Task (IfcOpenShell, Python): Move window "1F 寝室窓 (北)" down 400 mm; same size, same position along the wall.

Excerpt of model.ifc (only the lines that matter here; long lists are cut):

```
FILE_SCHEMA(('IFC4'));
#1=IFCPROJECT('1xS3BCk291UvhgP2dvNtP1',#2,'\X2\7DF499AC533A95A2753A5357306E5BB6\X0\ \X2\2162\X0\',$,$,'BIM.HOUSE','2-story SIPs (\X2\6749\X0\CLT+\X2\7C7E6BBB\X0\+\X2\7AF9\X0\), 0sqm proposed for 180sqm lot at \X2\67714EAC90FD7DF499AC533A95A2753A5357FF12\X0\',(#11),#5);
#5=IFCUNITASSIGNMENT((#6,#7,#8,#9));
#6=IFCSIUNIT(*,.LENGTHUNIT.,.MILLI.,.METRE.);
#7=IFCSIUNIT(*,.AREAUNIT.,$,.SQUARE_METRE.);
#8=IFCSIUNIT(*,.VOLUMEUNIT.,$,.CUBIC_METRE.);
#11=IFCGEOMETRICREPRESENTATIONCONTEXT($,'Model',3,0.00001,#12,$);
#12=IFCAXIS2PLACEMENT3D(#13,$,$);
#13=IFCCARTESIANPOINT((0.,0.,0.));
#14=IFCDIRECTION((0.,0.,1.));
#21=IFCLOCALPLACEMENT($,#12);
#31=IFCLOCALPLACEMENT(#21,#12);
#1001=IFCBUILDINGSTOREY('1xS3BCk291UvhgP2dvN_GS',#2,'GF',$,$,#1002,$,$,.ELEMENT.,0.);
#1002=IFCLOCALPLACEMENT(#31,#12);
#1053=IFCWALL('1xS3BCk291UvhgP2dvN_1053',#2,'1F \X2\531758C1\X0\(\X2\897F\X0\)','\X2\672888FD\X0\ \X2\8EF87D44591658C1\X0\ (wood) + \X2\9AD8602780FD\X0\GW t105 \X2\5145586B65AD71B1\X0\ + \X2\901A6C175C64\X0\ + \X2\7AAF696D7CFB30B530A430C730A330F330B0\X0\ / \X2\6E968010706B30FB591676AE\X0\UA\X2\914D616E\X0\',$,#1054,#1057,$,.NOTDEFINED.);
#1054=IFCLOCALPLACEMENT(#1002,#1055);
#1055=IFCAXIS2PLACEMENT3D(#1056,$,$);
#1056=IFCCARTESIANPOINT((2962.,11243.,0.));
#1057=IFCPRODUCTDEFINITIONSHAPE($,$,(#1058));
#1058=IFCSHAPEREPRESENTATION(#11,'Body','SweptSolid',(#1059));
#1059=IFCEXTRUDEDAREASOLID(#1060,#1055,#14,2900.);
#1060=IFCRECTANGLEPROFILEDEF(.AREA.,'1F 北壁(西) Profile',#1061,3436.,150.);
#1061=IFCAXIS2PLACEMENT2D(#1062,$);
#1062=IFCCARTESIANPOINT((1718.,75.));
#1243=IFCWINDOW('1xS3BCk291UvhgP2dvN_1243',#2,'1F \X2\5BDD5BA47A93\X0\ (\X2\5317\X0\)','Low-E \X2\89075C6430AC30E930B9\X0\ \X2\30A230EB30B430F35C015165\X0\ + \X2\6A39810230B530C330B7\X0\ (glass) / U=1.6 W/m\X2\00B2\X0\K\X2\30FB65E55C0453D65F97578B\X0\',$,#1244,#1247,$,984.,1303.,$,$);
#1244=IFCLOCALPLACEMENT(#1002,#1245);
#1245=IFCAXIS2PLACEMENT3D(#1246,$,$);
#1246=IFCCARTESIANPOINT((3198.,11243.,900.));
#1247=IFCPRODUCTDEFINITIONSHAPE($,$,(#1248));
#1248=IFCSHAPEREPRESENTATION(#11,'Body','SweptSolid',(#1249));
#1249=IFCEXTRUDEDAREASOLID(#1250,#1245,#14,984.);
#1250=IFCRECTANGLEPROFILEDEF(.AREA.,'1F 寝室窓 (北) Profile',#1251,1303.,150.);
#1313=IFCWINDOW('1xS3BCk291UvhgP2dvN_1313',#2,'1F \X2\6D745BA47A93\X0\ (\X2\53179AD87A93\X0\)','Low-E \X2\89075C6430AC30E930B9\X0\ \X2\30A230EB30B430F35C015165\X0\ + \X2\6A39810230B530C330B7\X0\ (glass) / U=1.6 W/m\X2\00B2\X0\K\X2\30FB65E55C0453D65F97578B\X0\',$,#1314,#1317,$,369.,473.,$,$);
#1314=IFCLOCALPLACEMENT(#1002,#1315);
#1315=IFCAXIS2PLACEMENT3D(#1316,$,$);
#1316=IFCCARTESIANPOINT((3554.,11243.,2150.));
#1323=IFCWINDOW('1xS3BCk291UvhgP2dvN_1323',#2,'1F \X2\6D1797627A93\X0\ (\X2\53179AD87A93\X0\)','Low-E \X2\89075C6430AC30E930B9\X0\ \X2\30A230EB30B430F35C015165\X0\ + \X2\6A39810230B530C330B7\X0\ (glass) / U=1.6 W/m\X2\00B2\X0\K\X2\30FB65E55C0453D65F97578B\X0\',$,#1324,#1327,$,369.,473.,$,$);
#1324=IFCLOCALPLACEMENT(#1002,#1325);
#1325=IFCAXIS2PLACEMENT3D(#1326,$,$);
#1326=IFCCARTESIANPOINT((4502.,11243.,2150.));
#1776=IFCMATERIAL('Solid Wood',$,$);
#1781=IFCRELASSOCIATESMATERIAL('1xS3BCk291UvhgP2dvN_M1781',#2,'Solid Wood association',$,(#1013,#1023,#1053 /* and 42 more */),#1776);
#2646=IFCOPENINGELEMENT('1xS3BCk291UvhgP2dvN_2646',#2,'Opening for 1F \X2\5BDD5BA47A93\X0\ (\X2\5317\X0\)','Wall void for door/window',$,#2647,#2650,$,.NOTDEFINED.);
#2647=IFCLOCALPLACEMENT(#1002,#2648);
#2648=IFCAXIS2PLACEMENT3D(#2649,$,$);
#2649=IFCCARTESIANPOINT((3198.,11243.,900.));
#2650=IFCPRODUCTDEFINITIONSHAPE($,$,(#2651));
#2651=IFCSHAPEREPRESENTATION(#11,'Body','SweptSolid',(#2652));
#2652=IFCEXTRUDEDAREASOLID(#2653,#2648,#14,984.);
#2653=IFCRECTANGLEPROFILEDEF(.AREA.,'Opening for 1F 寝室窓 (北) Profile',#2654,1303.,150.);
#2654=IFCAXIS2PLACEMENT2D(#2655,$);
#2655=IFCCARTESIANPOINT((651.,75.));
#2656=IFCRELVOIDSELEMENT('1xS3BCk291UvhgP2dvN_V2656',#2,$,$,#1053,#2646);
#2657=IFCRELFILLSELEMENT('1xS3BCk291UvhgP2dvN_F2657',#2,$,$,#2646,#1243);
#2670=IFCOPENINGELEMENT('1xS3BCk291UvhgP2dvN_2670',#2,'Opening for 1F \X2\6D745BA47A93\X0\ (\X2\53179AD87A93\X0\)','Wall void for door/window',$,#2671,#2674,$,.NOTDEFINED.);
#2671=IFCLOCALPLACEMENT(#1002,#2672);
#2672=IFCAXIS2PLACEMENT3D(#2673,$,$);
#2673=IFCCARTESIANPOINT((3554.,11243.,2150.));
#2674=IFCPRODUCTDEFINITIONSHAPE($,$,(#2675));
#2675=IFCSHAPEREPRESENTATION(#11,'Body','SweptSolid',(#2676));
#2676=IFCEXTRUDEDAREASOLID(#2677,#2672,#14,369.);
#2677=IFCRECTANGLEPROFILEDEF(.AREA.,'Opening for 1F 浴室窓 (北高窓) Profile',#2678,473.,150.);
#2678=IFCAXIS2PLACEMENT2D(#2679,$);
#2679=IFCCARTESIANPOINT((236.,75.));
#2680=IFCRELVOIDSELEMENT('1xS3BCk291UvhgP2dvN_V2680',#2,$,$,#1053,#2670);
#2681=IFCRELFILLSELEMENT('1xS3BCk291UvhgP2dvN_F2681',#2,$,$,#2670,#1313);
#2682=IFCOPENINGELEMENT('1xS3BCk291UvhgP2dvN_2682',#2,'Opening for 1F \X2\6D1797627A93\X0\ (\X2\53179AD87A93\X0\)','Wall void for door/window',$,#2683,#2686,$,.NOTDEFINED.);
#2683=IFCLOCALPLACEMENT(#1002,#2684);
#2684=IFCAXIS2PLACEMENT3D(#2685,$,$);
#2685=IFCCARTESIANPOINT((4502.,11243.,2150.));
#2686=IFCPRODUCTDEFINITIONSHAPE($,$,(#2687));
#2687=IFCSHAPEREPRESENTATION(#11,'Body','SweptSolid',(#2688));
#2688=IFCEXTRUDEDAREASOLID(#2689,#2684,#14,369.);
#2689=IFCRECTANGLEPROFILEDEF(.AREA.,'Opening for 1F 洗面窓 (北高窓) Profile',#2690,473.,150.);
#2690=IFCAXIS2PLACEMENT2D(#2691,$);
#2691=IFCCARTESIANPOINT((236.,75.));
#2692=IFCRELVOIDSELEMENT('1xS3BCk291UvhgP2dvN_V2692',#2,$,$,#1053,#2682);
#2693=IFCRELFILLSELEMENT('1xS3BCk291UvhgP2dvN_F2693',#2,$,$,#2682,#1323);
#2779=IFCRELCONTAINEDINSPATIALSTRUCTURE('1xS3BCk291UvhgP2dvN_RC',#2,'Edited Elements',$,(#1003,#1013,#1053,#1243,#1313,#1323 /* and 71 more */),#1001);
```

```python
import numpy as np
import ifcopenshell
import ifcopenshell.api.geometry
import ifcopenshell.util.placement
import ifcopenshell.util.unit

model = ifcopenshell.open("model.ifc")
unit_scale = ifcopenshell.util.unit.calculate_unit_scale(model)

window = model.by_id(1243)
opening = window.FillsVoids[0].RelatingOpeningElement
dz = -400.0

shift = np.array([0.0, 0.0, dz])
# The window is not placed relative to its opening, so move both.
for product in (opening, window):
    matrix = ifcopenshell.util.placement.get_local_placement(product.ObjectPlacement)
    matrix[:3, 3] += shift
    ifcopenshell.api.geometry.edit_object_placement(model, product=product, matrix=matrix, is_si=False)

print(f"moved by {dz * unit_scale:+.3f} m")

model.write("model_v2.ifc")
```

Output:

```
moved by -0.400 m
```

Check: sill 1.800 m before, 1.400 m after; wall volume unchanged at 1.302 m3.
